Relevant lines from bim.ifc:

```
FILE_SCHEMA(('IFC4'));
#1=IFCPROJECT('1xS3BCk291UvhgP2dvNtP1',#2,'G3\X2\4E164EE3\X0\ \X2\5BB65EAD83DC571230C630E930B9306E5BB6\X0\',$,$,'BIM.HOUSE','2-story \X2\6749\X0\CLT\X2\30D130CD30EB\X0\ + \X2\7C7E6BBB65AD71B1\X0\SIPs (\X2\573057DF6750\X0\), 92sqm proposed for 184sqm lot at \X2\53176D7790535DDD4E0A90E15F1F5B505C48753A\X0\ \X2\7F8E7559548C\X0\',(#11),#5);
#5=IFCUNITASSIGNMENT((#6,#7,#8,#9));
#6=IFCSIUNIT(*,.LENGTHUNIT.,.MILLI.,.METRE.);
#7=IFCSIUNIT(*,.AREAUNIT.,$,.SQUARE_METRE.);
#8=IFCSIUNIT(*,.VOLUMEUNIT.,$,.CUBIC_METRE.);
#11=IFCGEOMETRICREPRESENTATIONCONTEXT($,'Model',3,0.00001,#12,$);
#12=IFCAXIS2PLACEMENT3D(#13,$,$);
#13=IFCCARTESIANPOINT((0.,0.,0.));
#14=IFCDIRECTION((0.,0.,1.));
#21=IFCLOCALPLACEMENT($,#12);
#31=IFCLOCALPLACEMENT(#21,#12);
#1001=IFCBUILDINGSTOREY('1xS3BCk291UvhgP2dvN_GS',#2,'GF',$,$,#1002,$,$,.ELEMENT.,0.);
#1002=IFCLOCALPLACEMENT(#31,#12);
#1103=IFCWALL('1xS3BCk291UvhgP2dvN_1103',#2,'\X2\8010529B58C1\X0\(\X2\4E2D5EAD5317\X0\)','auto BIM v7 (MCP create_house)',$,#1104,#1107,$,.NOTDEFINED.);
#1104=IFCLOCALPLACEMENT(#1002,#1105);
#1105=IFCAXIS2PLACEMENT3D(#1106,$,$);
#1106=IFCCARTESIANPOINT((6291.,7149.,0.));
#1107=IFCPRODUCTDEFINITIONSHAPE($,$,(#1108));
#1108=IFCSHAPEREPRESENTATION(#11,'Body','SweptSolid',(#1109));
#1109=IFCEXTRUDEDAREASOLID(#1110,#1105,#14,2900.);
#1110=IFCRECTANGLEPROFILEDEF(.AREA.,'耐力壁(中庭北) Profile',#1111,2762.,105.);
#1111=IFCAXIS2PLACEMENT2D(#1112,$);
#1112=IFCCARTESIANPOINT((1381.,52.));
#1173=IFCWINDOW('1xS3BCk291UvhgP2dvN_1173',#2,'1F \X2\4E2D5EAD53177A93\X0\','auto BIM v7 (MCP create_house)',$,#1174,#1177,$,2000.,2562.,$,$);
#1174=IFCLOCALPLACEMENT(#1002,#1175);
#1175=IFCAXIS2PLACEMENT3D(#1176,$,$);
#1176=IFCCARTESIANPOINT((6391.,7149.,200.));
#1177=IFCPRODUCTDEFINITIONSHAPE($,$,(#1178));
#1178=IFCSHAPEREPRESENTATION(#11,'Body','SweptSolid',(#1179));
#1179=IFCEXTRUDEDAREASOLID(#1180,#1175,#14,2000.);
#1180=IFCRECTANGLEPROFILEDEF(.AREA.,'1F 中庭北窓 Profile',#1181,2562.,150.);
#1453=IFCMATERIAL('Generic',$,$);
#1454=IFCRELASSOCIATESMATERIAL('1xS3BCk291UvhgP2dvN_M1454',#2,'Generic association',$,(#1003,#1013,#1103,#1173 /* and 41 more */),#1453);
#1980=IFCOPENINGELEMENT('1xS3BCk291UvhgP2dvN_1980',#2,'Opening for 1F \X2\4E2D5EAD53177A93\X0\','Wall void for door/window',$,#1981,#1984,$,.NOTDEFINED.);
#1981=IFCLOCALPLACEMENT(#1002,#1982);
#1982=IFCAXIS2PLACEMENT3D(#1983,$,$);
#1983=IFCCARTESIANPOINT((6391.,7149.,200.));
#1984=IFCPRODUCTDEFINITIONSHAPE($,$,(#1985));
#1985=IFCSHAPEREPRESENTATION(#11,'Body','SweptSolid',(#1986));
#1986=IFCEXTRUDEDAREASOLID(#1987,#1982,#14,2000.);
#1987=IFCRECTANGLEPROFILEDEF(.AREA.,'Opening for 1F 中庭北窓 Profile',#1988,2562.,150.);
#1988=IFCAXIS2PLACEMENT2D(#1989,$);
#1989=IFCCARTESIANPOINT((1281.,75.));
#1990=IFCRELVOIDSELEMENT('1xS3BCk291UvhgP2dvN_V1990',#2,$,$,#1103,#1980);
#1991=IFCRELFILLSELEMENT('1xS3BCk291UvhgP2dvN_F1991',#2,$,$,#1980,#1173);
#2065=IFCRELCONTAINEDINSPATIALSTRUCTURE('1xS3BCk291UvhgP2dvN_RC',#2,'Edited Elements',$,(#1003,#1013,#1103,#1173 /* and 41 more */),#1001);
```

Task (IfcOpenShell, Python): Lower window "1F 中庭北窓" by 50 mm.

```python
import numpy as np
import ifcopenshell
import ifcopenshell.api.geometry
import ifcopenshell.util.placement
import ifcopenshell.util.unit

model = ifcopenshell.open("bim.ifc")
unit_scale = ifcopenshell.util.unit.calculate_unit_scale(model)

window = model.by_id(1173)
opening = window.FillsVoids[0].RelatingOpeningElement
dz = -50.0

shift = np.array([0.0, 0.0, dz])
# The window is not placed relative to its opening, so move both.
for product in (opening, window):
    matrix = ifcopenshell.util.placement.get_local_placement(product.ObjectPlacement)
    matrix[:3, 3] += shift
    ifcopenshell.api.geometry.edit_object_placement(model, product=product, matrix=matrix, is_si=False)

print(f"moved by {dz * unit_scale:+.3f} m")

model.write("bim_edited.ifc")
```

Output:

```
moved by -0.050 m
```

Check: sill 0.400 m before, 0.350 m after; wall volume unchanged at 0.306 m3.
